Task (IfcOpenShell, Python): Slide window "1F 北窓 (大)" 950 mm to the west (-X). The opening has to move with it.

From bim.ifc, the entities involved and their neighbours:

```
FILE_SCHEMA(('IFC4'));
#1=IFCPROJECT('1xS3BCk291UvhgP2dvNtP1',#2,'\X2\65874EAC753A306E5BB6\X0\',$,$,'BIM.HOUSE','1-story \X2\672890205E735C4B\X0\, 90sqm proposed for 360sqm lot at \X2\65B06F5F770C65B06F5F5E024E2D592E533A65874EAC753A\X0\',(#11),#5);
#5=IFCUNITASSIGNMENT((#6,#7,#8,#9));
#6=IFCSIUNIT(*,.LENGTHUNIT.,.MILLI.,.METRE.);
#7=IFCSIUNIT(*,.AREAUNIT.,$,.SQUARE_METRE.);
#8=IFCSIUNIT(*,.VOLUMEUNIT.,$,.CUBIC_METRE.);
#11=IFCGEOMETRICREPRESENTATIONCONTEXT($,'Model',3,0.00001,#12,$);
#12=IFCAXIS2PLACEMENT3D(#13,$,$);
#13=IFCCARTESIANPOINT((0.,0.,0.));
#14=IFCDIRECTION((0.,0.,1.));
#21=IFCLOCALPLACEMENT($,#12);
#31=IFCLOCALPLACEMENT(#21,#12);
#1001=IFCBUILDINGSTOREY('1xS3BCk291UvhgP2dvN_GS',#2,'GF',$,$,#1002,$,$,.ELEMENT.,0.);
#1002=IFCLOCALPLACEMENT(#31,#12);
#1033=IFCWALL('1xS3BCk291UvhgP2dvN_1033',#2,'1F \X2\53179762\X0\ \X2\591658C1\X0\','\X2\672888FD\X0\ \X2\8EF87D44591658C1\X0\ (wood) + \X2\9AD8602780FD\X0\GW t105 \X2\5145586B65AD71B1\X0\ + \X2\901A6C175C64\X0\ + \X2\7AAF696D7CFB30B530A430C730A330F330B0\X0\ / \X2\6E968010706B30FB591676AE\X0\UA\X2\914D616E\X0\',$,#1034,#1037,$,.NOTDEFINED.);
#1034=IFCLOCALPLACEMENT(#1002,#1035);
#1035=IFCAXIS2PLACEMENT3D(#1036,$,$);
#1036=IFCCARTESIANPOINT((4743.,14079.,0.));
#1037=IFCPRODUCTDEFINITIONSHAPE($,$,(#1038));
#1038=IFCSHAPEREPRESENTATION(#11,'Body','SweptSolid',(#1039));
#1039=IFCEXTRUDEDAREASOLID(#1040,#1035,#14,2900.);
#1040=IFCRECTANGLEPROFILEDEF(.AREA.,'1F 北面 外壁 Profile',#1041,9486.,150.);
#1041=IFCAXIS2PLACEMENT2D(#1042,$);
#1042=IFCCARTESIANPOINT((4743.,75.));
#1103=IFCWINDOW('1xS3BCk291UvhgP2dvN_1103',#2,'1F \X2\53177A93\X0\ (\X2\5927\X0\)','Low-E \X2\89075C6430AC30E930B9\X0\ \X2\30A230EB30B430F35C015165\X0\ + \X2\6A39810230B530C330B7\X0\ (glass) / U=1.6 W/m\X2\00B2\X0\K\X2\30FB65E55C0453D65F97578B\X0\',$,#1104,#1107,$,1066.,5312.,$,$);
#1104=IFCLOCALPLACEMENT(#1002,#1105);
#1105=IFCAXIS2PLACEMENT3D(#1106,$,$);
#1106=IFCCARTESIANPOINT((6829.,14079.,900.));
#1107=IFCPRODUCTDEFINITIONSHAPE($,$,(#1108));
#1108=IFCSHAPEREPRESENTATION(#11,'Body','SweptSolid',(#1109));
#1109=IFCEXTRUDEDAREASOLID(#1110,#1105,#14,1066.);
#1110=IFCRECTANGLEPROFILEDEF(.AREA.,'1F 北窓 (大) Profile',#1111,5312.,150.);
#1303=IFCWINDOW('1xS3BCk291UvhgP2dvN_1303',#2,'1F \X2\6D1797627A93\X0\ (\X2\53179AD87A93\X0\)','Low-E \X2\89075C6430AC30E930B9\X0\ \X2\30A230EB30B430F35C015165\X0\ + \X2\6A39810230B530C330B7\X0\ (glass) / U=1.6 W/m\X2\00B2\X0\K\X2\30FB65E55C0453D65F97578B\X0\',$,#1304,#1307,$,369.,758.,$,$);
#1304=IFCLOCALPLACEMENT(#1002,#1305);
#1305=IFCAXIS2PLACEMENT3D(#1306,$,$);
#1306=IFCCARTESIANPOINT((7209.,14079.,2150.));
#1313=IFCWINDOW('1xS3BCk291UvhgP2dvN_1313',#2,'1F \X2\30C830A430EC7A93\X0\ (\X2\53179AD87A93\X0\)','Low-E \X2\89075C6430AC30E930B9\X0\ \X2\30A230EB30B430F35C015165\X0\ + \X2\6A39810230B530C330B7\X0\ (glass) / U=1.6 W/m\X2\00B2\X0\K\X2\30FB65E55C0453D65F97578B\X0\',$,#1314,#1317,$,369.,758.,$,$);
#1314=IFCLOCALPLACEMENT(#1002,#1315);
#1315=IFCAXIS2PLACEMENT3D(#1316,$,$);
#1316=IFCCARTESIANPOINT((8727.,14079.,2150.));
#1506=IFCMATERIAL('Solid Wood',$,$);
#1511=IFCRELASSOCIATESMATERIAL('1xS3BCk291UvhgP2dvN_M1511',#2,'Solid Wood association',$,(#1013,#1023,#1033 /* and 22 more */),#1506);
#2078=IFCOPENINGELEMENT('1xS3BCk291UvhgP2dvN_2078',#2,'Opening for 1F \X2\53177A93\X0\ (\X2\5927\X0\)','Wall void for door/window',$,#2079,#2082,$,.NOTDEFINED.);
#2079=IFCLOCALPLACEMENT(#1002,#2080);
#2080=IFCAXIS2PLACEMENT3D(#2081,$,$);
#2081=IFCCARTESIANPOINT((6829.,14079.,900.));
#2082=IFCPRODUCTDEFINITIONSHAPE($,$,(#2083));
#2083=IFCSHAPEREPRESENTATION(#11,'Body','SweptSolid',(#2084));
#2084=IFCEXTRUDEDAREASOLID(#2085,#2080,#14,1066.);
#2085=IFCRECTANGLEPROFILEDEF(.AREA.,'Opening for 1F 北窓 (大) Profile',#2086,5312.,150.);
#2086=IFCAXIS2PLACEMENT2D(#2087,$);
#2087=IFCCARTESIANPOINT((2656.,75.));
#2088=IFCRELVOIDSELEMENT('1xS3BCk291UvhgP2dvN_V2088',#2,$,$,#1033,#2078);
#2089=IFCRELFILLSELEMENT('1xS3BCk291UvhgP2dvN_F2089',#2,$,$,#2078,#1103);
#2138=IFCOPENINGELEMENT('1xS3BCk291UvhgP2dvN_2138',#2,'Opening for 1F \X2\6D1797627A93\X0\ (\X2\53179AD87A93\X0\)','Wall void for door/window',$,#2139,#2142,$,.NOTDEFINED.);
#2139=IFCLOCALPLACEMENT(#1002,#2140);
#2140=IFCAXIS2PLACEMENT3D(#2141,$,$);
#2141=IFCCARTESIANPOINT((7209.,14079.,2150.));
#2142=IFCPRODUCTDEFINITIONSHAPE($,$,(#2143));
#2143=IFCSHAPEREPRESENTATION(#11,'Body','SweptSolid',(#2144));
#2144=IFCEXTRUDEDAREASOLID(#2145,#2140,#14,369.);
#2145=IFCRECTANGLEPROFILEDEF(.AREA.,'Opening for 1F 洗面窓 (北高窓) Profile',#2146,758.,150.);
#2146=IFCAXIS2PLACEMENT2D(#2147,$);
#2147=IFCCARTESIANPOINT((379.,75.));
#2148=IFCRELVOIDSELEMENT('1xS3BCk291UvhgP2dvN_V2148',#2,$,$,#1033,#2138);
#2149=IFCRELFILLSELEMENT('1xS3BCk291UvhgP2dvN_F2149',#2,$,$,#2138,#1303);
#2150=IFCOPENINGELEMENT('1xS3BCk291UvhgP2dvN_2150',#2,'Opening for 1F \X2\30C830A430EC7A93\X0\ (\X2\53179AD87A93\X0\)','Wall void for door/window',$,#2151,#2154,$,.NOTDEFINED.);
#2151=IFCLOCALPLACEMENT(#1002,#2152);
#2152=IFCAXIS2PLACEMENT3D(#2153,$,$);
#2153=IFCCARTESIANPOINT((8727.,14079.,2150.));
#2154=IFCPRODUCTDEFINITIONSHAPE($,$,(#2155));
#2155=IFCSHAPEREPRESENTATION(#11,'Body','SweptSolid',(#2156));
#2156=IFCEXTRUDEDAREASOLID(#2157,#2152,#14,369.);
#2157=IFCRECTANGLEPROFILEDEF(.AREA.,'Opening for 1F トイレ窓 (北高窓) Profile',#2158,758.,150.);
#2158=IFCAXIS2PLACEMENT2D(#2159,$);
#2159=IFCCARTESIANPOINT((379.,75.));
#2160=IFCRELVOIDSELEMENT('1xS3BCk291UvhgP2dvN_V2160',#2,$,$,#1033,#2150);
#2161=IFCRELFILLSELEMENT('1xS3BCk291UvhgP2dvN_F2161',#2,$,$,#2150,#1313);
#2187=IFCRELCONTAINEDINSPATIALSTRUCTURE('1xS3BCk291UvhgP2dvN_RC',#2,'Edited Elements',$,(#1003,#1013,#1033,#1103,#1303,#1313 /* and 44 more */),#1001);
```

```python
import ifcopenshell
import ifcopenshell.api.geometry
import ifcopenshell.util.placement

model = ifcopenshell.open("bim.ifc")

window = model.by_guid("1xS3BCk291UvhgP2dvN_1103")
opening = window.FillsVoids[0].RelatingOpeningElement
wall = opening.VoidsElements[0].RelatingBuildingElement

wall_matrix = ifcopenshell.util.placement.get_local_placement(wall.ObjectPlacement)
shift = wall_matrix[:3, 0] * -950.0
before = ifcopenshell.util.placement.get_local_placement(window.ObjectPlacement)[:3, 3].copy()

# The window is not placed relative to its opening, so move both.
for product in (opening, window):
    matrix = ifcopenshell.util.placement.get_local_placement(product.ObjectPlacement)
    matrix[:3, 3] += shift
    ifcopenshell.api.geometry.edit_object_placement(model, product=product, matrix=matrix, is_si=False)

after = ifcopenshell.util.placement.get_local_placement(window.ObjectPlacement)[:3, 3]
print("window moved by", (after - before).round(3) + 0.0)

model.write("bim_rev.ifc")
```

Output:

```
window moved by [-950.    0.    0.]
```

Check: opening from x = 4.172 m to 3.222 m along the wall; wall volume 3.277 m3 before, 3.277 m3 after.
